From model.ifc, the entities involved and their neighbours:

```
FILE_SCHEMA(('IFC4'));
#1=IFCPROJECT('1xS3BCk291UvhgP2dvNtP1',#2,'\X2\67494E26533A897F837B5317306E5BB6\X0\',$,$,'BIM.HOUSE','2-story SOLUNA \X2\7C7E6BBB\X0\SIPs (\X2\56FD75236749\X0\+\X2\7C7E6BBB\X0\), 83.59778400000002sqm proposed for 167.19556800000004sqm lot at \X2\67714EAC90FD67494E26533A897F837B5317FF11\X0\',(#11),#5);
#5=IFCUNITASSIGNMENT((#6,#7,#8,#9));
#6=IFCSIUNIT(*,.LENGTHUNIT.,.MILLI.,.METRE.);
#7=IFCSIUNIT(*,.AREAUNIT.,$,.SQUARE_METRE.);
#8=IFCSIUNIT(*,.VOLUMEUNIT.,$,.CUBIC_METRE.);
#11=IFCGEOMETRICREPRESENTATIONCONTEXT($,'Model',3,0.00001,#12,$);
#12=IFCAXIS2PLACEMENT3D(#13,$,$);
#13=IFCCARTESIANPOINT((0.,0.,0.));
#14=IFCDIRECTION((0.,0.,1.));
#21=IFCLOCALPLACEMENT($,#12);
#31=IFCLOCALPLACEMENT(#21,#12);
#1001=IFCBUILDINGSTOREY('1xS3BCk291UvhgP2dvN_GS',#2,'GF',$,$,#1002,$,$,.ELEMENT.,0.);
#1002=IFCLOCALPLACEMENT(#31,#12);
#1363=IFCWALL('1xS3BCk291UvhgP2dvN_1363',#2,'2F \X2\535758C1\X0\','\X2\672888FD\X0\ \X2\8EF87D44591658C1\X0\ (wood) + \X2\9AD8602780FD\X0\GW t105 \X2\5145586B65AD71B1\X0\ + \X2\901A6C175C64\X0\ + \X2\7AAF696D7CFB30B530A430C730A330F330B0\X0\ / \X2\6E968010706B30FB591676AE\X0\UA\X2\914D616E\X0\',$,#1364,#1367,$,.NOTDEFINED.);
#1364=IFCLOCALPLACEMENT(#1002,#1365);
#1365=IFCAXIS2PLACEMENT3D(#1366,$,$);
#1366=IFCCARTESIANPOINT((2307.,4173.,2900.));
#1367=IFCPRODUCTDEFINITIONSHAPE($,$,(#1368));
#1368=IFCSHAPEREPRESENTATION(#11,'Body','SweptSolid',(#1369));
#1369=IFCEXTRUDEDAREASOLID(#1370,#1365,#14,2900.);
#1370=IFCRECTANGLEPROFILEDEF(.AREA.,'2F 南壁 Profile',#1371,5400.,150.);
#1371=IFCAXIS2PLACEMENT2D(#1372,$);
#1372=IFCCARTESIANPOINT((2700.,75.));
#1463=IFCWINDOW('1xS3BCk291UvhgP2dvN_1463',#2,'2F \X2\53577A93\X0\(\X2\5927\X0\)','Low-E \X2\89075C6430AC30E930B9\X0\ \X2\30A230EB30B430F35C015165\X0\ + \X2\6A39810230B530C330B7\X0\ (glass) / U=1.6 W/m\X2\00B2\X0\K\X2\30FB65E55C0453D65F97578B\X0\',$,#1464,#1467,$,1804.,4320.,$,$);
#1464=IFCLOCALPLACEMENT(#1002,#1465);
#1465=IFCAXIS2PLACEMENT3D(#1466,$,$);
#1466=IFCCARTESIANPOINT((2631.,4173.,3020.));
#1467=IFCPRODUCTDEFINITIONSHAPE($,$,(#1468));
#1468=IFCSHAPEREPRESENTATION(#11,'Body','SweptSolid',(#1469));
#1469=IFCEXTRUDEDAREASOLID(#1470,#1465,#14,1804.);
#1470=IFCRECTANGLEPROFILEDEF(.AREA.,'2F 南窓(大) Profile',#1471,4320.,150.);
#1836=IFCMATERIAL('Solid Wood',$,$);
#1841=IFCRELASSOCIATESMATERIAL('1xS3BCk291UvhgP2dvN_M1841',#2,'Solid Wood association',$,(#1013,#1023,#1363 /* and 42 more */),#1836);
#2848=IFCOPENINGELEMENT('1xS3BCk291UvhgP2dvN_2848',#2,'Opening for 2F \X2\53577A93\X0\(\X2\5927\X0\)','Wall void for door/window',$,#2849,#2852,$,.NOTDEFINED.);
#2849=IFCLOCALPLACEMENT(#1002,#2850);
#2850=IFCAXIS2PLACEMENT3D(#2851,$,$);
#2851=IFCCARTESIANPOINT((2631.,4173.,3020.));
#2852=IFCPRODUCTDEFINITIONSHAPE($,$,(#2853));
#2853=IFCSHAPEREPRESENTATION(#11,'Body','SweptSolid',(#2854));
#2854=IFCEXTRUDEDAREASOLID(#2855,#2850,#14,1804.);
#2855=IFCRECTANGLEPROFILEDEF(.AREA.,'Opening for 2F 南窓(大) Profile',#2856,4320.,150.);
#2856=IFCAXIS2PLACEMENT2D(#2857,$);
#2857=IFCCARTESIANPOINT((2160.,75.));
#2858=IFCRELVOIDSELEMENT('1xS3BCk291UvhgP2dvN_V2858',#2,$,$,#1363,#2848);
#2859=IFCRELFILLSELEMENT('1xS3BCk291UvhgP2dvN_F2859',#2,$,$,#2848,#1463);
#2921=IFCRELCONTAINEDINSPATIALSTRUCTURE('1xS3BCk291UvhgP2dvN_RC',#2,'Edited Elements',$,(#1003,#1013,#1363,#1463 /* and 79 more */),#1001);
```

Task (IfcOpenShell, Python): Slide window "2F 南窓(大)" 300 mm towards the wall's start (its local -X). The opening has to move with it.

```python
import ifcopenshell
import ifcopenshell.api.geometry
import ifcopenshell.util.placement
import ifcopenshell.util.unit

model = ifcopenshell.open("model.ifc")
unit_scale = ifcopenshell.util.unit.calculate_unit_scale(model)

window = model.by_guid("1xS3BCk291UvhgP2dvN_1463")
opening = window.FillsVoids[0].RelatingOpeningElement
wall = opening.VoidsElements[0].RelatingBuildingElement

wall_matrix = ifcopenshell.util.placement.get_local_placement(wall.ObjectPlacement)
shift = wall_matrix[:3, 0] * -0.3 / unit_scale
before = ifcopenshell.util.placement.get_local_placement(window.ObjectPlacement)[:3, 3].copy()

# The window is not placed relative to its opening, so move both.
for product in (opening, window):
    matrix = ifcopenshell.util.placement.get_local_placement(product.ObjectPlacement)
    matrix[:3, 3] += shift
    ifcopenshell.api.geometry.edit_object_placement(model, product=product, matrix=matrix, is_si=False)

after = ifcopenshell.util.placement.get_local_placement(window.ObjectPlacement)[:3, 3]
print("window moved by", (after - before).round(3) + 0.0)

model.write("model-out.ifc")
```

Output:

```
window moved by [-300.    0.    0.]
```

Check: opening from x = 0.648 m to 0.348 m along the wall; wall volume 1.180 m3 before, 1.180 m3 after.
